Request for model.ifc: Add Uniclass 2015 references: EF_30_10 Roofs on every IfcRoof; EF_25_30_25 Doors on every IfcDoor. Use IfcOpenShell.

First a look at what the model holds.

```python
import ifcopenshell

model = ifcopenshell.open("model.ifc")
print(model.schema)
print("classifications:", [c.Name for c in model.by_type("IfcClassification")])
for ifc_class in ("IfcDoor", "IfcRoof", "IfcStair", "IfcWall", "IfcWindow"):
    print(ifc_class, len(model.by_type(ifc_class)))
```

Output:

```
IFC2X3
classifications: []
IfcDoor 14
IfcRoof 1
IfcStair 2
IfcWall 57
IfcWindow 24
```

```python
import ifcopenshell
import ifcopenshell.api.classification

model = ifcopenshell.open("model.ifc")

# IFC2X3 requires Source and Edition and has no link from the project to the system.
system = model.create_entity("IfcClassification", Source="NBS", Edition="2015", Name="Uniclass 2015")

codes = {
    "IfcRoof": ("EF_30_10", "Roofs"),
    "IfcDoor": ("EF_25_30_25", "Doors"),
}
for ifc_class, (code, name) in codes.items():
    products = model.by_type(ifc_class)
    ifcopenshell.api.classification.add_reference(
        model, products=products, classification=system, identification=code, name=name
    )
    print(code, len(products))

model.write("model-out.ifc")
```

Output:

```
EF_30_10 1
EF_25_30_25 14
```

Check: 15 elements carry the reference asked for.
